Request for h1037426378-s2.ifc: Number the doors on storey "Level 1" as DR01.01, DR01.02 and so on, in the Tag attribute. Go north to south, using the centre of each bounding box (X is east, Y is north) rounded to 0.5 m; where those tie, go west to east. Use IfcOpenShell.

First a look at what the model holds.

```python
import ifcopenshell
import ifcopenshell.util.element
import ifcopenshell.util.placement

model = ifcopenshell.open("h1037426378-s2.ifc")
print(model.schema)
storey = next(s for s in model.by_type("IfcBuildingStorey") if s.Name == "Level 1")
doors = [e for e in ifcopenshell.util.element.get_decomposition(storey) if e.is_a("IfcDoor")]
for e in sorted(doors, key=lambda e: e.id()):
    origin = ifcopenshell.util.placement.get_local_placement(e.ObjectPlacement)[:3, 3]
    print(e.id(), e.Tag, e.Name, origin.round(2) + 0.0, sep=" | ")
```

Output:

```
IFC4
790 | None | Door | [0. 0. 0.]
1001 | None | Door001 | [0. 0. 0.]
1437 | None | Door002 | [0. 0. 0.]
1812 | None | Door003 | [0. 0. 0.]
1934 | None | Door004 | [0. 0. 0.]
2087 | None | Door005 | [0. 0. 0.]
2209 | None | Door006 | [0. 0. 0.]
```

```python
import ifcopenshell
import ifcopenshell.geom
import ifcopenshell.util.element
import ifcopenshell.util.shape

model = ifcopenshell.open("h1037426378-s2.ifc")
settings = ifcopenshell.geom.settings()
settings.set("use-world-coords", True)


def centre(element):
    shape = ifcopenshell.geom.create_shape(settings, element)
    return ifcopenshell.util.shape.get_bbox_centroid(shape.geometry)


storey = next(s for s in model.by_type("IfcBuildingStorey") if s.Name == "Level 1")
doors = [e for e in ifcopenshell.util.element.get_decomposition(storey) if e.is_a("IfcDoor")]

# Insertion points can sit at a corner or the storey origin, so sort by the geometry (in metres).
centres = {e: centre(e) for e in doors}
doors.sort(key=lambda e: (-round(centres[e][1] / 0.5), centres[e][0]))

for i, e in enumerate(doors, start=1):
    number = f"DR01.{i:02d}"
    e.Tag = number
    print(e.id(), number)

model.write("h1037426378-s2_updated.ifc")
```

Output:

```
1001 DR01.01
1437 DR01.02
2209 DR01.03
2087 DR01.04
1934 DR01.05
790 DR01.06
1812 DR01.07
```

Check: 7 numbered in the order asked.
